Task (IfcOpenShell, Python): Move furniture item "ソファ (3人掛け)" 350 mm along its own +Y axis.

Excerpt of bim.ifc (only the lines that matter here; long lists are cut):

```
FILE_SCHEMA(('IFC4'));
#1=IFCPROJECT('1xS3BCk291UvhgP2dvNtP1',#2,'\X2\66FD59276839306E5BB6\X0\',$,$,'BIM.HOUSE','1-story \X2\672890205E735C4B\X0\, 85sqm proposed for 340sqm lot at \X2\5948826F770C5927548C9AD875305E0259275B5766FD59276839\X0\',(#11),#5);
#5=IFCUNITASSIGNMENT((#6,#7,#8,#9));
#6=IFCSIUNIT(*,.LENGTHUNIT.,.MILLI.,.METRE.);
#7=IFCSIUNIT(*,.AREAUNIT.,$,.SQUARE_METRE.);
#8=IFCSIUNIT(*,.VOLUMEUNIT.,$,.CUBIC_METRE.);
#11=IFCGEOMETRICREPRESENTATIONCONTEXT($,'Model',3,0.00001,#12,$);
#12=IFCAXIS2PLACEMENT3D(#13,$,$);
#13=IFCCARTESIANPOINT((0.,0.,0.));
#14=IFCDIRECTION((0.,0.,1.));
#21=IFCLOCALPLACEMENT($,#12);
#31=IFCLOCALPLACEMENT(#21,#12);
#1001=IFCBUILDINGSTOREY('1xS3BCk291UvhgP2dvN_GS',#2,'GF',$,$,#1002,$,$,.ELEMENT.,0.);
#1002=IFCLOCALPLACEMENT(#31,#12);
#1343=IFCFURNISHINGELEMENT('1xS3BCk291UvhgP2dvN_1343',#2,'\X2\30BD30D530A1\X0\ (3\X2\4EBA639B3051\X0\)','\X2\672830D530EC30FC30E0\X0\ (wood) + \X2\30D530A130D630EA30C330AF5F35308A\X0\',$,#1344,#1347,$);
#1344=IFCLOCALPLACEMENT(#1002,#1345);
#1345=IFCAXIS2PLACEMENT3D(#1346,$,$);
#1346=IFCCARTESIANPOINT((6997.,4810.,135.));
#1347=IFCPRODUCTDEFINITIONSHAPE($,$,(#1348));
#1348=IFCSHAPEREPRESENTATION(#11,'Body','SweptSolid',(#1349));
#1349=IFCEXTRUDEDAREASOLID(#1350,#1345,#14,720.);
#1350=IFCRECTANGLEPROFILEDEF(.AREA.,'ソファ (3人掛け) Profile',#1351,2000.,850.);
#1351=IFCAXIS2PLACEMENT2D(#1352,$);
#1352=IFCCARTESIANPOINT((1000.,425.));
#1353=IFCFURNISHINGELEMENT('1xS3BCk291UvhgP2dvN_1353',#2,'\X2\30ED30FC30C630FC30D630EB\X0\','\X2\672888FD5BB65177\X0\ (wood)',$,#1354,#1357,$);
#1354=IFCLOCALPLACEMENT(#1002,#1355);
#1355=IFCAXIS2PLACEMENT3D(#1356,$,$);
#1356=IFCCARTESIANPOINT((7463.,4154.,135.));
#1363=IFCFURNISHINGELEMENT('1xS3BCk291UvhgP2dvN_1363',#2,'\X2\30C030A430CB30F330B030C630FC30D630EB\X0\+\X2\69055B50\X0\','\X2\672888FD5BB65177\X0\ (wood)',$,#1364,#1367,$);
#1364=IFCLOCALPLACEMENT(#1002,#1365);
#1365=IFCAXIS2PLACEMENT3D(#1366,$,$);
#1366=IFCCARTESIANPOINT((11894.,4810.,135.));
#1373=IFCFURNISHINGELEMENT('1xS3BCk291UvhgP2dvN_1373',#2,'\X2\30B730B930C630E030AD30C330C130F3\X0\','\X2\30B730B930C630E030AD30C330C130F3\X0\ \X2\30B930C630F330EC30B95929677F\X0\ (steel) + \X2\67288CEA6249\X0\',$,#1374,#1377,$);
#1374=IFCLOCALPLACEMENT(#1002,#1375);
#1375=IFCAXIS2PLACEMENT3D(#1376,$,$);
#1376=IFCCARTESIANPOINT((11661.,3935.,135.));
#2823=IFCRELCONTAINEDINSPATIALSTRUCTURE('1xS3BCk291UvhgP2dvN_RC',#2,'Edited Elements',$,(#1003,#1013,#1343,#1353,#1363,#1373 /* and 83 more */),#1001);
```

```python
import ifcopenshell
import ifcopenshell.api.geometry
import ifcopenshell.util.placement
import ifcopenshell.util.unit

model = ifcopenshell.open("bim.ifc")
unit_scale = ifcopenshell.util.unit.calculate_unit_scale(model)

item = model.by_id(1343)
matrix = ifcopenshell.util.placement.get_local_placement(item.ObjectPlacement)
matrix[:3, 3] += matrix[:3, 1] * 0.35 / unit_scale
ifcopenshell.api.geometry.edit_object_placement(model, product=item, matrix=matrix, is_si=False)

print(ifcopenshell.util.placement.get_local_placement(item.ObjectPlacement).round(3) + 0.0)

model.write("bim-out.ifc")
```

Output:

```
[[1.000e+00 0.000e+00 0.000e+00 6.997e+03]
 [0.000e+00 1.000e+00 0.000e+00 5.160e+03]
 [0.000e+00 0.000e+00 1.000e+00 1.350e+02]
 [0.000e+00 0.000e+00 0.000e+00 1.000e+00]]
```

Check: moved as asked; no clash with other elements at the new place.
